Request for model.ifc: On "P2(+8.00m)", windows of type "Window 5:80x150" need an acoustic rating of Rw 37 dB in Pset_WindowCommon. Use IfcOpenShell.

First a look at what the model holds.

```python
import ifcopenshell
import ifcopenshell.util.element

model = ifcopenshell.open("model.ifc")
print(model.schema)
storey = next(s for s in model.by_type("IfcBuildingStorey") if s.Name == "P2(+8.00m)")
windows = [e for e in ifcopenshell.util.element.get_decomposition(storey) if e.is_a("IfcWindow")]
seen = {}
for e in windows:
    element_type = ifcopenshell.util.element.get_type(e)
    key = (element_type.Name if element_type != e and element_type else None, ifcopenshell.util.element.get_pset(e, "Pset_WindowCommon", "AcousticRating"))
    seen[key] = seen.get(key, 0) + 1
for (name, value), count in sorted(seen.items(), key=str):
    print(count, "x", name, "|", value)
```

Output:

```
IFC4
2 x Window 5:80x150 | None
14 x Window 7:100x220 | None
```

```python
import ifcopenshell
import ifcopenshell.api.pset
import ifcopenshell.util.element

model = ifcopenshell.open("model.ifc")

storey = next(s for s in model.by_type("IfcBuildingStorey") if s.Name == "P2(+8.00m)")
windows = [e for e in ifcopenshell.util.element.get_decomposition(storey) if e.is_a("IfcWindow")]

count = 0
for e in windows:
    element_type = ifcopenshell.util.element.get_type(e)
    if element_type in (None, e) or element_type.Name != "Window 5:80x150":
        continue
    # add_pset returns the element's existing set when there is one.
    pset = ifcopenshell.api.pset.add_pset(model, product=e, name="Pset_WindowCommon")
    ifcopenshell.api.pset.edit_pset(model, pset=pset, properties={"AcousticRating": "Rw 37 dB"})
    count += 1

print(count, "windows updated")

model.write("model-out.ifc")
```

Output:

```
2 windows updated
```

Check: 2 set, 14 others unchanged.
